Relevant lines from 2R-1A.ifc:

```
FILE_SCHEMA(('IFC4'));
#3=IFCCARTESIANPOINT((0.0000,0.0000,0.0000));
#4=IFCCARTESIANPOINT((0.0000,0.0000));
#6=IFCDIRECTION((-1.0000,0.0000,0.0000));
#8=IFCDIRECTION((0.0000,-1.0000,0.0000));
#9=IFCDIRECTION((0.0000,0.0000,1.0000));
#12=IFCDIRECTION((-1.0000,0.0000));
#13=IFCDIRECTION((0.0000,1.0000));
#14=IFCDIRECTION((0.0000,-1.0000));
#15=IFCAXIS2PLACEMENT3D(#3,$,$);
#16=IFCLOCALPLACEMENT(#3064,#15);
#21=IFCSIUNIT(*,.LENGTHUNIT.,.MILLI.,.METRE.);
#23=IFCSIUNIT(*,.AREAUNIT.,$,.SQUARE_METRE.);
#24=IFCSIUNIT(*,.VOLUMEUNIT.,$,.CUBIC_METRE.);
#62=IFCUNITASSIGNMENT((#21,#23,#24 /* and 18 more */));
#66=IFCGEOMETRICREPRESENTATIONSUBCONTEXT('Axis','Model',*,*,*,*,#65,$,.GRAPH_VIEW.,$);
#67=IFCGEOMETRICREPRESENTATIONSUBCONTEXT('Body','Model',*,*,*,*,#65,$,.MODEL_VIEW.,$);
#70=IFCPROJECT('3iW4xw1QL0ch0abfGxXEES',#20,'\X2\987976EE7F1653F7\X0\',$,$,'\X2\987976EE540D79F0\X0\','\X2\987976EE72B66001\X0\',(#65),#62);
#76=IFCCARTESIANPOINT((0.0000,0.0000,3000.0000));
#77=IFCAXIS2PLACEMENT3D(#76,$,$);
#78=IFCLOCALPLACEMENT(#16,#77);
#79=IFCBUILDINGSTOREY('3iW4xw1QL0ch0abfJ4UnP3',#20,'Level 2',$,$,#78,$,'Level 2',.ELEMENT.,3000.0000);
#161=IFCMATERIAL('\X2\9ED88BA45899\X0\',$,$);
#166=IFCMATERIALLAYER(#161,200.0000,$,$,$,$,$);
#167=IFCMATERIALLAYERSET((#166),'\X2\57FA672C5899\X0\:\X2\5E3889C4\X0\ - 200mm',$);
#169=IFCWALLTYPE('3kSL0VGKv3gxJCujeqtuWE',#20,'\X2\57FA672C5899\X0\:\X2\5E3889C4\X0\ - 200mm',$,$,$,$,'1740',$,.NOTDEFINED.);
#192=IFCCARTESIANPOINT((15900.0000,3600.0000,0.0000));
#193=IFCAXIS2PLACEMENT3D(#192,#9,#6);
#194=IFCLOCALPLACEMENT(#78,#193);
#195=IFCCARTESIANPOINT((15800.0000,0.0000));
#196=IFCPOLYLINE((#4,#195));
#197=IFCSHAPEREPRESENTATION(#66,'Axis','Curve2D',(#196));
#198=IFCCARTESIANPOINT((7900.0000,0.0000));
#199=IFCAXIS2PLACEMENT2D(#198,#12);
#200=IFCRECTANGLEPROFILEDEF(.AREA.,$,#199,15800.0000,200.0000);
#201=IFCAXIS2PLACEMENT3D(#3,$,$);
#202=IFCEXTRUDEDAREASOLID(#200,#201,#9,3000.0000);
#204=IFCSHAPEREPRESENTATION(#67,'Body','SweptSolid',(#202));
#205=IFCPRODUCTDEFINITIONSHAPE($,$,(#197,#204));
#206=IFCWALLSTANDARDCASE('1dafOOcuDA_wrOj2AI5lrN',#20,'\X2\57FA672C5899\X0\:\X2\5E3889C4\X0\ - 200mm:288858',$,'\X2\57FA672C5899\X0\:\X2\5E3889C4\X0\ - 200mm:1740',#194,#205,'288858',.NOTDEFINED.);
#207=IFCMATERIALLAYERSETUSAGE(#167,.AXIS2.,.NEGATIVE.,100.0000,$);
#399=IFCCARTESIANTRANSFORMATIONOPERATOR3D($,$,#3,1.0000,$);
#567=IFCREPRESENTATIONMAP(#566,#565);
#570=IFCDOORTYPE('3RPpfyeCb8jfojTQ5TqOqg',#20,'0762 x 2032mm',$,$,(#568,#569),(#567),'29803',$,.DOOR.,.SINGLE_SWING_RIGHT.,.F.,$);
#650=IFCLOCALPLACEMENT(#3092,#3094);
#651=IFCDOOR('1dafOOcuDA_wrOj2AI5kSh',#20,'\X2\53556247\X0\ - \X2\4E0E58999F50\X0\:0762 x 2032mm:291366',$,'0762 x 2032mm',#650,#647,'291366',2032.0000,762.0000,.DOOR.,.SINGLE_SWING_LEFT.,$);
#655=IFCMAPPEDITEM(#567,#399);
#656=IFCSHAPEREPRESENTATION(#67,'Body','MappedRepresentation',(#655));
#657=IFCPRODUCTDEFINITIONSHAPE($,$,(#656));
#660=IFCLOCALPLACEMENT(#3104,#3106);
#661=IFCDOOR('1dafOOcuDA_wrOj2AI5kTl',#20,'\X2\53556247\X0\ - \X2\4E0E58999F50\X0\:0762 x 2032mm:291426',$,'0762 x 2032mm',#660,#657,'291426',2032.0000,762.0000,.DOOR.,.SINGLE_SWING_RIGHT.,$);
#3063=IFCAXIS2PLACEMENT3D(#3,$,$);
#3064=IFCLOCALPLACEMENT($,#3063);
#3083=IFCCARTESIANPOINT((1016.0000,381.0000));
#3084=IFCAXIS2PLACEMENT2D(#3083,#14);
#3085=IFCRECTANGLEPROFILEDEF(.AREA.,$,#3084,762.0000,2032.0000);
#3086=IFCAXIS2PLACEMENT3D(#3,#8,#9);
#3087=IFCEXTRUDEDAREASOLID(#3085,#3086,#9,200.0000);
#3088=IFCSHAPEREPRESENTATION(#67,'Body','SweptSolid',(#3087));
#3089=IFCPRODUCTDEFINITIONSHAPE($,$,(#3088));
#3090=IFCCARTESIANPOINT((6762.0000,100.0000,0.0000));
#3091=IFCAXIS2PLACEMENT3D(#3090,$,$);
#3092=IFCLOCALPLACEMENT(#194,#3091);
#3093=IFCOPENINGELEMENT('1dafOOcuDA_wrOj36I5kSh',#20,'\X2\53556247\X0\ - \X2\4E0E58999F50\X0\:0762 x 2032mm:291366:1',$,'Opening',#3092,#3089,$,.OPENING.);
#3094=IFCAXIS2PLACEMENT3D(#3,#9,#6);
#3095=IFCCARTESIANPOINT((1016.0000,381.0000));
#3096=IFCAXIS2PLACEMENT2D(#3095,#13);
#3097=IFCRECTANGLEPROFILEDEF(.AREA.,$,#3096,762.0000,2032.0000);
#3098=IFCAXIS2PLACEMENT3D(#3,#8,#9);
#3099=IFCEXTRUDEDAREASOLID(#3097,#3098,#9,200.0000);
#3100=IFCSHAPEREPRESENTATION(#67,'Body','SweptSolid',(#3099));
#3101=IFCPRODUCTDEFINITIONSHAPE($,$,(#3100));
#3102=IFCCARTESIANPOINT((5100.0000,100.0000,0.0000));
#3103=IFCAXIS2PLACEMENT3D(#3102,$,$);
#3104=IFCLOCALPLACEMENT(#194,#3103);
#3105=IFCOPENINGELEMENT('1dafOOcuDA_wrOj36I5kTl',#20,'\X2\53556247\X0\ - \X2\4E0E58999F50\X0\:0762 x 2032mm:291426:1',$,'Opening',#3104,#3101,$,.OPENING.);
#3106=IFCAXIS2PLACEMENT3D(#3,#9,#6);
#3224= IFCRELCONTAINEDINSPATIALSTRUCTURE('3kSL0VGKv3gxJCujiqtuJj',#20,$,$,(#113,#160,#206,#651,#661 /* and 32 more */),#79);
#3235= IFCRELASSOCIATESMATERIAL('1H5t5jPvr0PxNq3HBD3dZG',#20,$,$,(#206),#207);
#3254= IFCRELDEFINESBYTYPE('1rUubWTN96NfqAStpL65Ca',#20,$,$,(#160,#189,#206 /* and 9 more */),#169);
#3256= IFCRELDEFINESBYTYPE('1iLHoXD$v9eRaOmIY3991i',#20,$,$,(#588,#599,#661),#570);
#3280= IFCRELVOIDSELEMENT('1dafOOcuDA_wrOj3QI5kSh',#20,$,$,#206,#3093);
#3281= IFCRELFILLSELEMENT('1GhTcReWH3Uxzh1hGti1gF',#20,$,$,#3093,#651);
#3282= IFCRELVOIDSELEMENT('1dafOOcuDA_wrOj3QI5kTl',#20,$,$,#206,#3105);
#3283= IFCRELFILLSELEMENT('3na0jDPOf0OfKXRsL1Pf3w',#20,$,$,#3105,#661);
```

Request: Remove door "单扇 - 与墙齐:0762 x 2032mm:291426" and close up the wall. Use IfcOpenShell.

```python
import ifcopenshell
import ifcopenshell.api.feature
import ifcopenshell.api.root
import ifcopenshell.geom
import ifcopenshell.util.shape

model = ifcopenshell.open("2R-1A.ifc")
settings = ifcopenshell.geom.settings()


def volume(element):
    """Net volume in cubic metres, openings subtracted."""
    shape = ifcopenshell.geom.create_shape(settings, element)
    return ifcopenshell.util.shape.get_volume(shape.geometry)


door = model.by_guid("1dafOOcuDA_wrOj2AI5kTl")
opening = door.FillsVoids[0].RelatingOpeningElement
wall = opening.VoidsElements[0].RelatingBuildingElement
before = volume(wall)

ifcopenshell.api.root.remove_product(model, product=door)
ifcopenshell.api.feature.remove_feature(model, feature=opening)

after = volume(wall)

print(f"wall volume {before:.3f} -> {after:.3f} m3")

model.write("2R-1A_v2.ifc")
```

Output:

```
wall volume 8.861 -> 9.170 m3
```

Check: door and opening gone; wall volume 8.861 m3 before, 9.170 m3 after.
